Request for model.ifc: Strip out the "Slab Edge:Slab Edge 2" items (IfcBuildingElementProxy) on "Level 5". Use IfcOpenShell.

First a look at what the model holds.

```python
import ifcopenshell
import ifcopenshell.util.element

model = ifcopenshell.open("model.ifc")
print(model.schema)
storey = next(s for s in model.by_type("IfcBuildingStorey") if s.Name == "Level 5")
proxies = [e for e in ifcopenshell.util.element.get_decomposition(storey) if e.is_a("IfcBuildingElementProxy")]
seen = {}
for e in proxies:
    element_type = ifcopenshell.util.element.get_type(e)
    name = element_type.Name if element_type not in (None, e) else None
    seen[name] = seen.get(name, 0) + 1
for name, count in sorted(seen.items(), key=str):
    print(count, "x", name)
```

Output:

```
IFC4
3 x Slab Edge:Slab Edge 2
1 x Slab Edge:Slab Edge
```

```python
import ifcopenshell
import ifcopenshell.api.root
import ifcopenshell.util.element

model = ifcopenshell.open("model.ifc")

storey = next(s for s in model.by_type("IfcBuildingStorey") if s.Name == "Level 5")
proxies = [e for e in ifcopenshell.util.element.get_decomposition(storey) if e.is_a("IfcBuildingElementProxy")]
targets = [e for e in proxies if (t := ifcopenshell.util.element.get_type(e)) not in (None, e) and t.Name == "Slab Edge:Slab Edge 2"]

for e in targets:
    ifcopenshell.api.root.remove_product(model, product=e)
print(len(targets), "removed")

model.write("model_edited.ifc")
```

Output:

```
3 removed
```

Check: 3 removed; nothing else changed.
